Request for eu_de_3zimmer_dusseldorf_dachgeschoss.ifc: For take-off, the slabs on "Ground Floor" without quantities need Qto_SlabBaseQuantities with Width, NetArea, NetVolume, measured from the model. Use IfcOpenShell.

First a look at what the model holds.

```python
import ifcopenshell
import ifcopenshell.util.element
import ifcopenshell.util.unit

model = ifcopenshell.open("eu_de_3zimmer_dusseldorf_dachgeschoss.ifc")
print(model.schema)
for unit_type in ("LENGTHUNIT", "AREAUNIT", "VOLUMEUNIT"):
    print(unit_type, ifcopenshell.util.unit.calculate_unit_scale(model, unit_type))
storey = next(s for s in model.by_type("IfcBuildingStorey") if s.Name == "Ground Floor")
slabs = [e for e in ifcopenshell.util.element.get_decomposition(storey) if e.is_a("IfcSlab")]
for e in sorted(slabs, key=lambda e: e.id()):
    print(e.id(), e.is_a(), e.Name, list(ifcopenshell.util.element.get_psets(e, qtos_only=True)), sep=" | ")
```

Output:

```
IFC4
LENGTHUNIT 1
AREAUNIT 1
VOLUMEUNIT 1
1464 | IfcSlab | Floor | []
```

```python
import ifcopenshell
import ifcopenshell.api.pset
import ifcopenshell.geom
import ifcopenshell.util.element
import ifcopenshell.util.shape
import ifcopenshell.util.unit

model = ifcopenshell.open("eu_de_3zimmer_dusseldorf_dachgeschoss.ifc")
unit_scale = ifcopenshell.util.unit.calculate_unit_scale(model)
area_scale = ifcopenshell.util.unit.calculate_unit_scale(model, "AREAUNIT")
volume_scale = ifcopenshell.util.unit.calculate_unit_scale(model, "VOLUMEUNIT")
settings = ifcopenshell.geom.settings()

storey = next(s for s in model.by_type("IfcBuildingStorey") if s.Name == "Ground Floor")
slabs = [e for e in ifcopenshell.util.element.get_decomposition(storey) if e.is_a("IfcSlab")]

for e in sorted(slabs, key=lambda e: e.id()):
    if ifcopenshell.util.element.get_psets(e, qtos_only=True, should_inherit=False):
        continue
    # Geometry comes back in metres, in the element's own axes.
    shape = ifcopenshell.geom.create_shape(settings, e)
    values = {
        "Width": ifcopenshell.util.shape.get_z(shape.geometry) / unit_scale,
        "NetArea": ifcopenshell.util.shape.get_footprint_area(shape.geometry) / area_scale,
        "NetVolume": ifcopenshell.util.shape.get_volume(shape.geometry) / volume_scale,
    }
    qto = ifcopenshell.api.pset.add_qto(model, product=e, name="Qto_SlabBaseQuantities")
    ifcopenshell.api.pset.edit_qto(model, qto=qto, properties=values)
    print(e.id(), {k: round(v, 3) for k, v in values.items()})

model.write("eu_de_3zimmer_dusseldorf_dachgeschoss_edited.ifc")
```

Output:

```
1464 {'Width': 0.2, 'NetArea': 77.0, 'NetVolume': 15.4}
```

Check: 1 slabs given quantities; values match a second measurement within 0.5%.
